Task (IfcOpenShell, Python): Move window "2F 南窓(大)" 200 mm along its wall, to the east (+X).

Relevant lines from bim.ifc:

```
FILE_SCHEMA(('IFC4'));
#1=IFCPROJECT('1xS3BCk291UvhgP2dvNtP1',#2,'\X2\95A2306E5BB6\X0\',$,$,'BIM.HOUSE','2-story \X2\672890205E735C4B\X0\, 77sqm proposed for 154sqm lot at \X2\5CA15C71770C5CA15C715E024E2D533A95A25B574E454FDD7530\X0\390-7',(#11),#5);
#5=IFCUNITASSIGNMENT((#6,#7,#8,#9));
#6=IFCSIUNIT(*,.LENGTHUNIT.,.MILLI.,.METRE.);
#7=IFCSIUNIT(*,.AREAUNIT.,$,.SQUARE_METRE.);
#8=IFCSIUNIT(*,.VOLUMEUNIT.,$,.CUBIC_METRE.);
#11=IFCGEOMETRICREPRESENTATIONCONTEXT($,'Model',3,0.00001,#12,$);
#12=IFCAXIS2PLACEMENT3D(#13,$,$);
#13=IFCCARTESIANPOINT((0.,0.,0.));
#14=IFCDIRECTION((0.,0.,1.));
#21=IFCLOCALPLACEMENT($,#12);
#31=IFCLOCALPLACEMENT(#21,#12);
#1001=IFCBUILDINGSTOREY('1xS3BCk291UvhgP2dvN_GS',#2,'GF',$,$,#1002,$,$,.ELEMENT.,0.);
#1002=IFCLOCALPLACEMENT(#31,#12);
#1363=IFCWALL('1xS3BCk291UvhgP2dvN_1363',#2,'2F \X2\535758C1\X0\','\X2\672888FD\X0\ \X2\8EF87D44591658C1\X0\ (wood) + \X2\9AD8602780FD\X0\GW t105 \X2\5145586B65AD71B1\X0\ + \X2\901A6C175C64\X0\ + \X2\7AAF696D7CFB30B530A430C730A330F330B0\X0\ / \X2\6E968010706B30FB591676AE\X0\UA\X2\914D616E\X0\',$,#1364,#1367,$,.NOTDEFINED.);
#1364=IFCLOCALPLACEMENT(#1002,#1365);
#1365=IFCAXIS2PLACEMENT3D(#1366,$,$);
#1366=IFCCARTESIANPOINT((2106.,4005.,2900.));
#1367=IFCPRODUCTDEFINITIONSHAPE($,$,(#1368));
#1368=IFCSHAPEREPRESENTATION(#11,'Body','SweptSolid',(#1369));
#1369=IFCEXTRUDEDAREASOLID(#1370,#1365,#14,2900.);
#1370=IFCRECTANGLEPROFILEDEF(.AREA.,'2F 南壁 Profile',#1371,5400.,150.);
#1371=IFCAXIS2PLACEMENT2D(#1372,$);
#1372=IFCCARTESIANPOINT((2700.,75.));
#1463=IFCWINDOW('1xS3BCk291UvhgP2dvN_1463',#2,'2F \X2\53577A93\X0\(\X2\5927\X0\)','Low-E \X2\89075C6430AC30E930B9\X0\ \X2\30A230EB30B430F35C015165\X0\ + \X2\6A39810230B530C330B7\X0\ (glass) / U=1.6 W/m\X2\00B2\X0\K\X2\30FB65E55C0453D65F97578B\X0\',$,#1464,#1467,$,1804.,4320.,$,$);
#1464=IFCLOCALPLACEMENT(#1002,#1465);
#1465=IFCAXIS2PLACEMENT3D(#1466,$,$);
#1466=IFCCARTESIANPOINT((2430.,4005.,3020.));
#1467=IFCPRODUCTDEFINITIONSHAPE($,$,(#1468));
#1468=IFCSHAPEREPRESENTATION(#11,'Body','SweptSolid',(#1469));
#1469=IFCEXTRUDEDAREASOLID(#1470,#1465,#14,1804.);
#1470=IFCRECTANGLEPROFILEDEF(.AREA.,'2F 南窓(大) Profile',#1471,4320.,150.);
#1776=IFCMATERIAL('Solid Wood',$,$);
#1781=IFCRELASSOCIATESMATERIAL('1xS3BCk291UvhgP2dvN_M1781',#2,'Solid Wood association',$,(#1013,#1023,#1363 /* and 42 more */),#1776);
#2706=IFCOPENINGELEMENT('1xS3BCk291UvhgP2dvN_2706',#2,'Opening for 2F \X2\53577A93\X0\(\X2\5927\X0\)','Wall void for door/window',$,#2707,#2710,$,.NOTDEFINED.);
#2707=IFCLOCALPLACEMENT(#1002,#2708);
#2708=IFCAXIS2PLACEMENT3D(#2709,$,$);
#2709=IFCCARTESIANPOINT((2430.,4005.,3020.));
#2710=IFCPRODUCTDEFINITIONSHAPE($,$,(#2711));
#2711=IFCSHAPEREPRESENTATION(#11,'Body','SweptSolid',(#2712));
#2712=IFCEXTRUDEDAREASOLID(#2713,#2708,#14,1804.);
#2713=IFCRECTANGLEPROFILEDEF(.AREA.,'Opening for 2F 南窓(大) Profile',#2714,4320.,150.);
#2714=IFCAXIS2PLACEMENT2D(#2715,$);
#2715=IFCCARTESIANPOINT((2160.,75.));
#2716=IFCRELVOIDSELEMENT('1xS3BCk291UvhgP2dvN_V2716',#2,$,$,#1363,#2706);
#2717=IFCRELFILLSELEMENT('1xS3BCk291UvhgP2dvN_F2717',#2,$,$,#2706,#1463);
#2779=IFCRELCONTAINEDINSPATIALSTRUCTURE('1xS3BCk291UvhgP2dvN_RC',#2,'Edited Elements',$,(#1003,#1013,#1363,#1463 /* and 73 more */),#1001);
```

```python
import ifcopenshell
import ifcopenshell.api.geometry
import ifcopenshell.util.placement
import ifcopenshell.util.unit

model = ifcopenshell.open("bim.ifc")
unit_scale = ifcopenshell.util.unit.calculate_unit_scale(model)

window = model.by_id(1463)
opening = window.FillsVoids[0].RelatingOpeningElement
wall = opening.VoidsElements[0].RelatingBuildingElement

wall_matrix = ifcopenshell.util.placement.get_local_placement(wall.ObjectPlacement)
shift = wall_matrix[:3, 0] * 0.2 / unit_scale
before = ifcopenshell.util.placement.get_local_placement(window.ObjectPlacement)[:3, 3].copy()

# The window is not placed relative to its opening, so move both.
for product in (opening, window):
    matrix = ifcopenshell.util.placement.get_local_placement(product.ObjectPlacement)
    matrix[:3, 3] += shift
    ifcopenshell.api.geometry.edit_object_placement(model, product=product, matrix=matrix, is_si=False)

after = ifcopenshell.util.placement.get_local_placement(window.ObjectPlacement)[:3, 3]
print("window moved by", (after - before).round(3) + 0.0)

model.write("bim_updated.ifc")
```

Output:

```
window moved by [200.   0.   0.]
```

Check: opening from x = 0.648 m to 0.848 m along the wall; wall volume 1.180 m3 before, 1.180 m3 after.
